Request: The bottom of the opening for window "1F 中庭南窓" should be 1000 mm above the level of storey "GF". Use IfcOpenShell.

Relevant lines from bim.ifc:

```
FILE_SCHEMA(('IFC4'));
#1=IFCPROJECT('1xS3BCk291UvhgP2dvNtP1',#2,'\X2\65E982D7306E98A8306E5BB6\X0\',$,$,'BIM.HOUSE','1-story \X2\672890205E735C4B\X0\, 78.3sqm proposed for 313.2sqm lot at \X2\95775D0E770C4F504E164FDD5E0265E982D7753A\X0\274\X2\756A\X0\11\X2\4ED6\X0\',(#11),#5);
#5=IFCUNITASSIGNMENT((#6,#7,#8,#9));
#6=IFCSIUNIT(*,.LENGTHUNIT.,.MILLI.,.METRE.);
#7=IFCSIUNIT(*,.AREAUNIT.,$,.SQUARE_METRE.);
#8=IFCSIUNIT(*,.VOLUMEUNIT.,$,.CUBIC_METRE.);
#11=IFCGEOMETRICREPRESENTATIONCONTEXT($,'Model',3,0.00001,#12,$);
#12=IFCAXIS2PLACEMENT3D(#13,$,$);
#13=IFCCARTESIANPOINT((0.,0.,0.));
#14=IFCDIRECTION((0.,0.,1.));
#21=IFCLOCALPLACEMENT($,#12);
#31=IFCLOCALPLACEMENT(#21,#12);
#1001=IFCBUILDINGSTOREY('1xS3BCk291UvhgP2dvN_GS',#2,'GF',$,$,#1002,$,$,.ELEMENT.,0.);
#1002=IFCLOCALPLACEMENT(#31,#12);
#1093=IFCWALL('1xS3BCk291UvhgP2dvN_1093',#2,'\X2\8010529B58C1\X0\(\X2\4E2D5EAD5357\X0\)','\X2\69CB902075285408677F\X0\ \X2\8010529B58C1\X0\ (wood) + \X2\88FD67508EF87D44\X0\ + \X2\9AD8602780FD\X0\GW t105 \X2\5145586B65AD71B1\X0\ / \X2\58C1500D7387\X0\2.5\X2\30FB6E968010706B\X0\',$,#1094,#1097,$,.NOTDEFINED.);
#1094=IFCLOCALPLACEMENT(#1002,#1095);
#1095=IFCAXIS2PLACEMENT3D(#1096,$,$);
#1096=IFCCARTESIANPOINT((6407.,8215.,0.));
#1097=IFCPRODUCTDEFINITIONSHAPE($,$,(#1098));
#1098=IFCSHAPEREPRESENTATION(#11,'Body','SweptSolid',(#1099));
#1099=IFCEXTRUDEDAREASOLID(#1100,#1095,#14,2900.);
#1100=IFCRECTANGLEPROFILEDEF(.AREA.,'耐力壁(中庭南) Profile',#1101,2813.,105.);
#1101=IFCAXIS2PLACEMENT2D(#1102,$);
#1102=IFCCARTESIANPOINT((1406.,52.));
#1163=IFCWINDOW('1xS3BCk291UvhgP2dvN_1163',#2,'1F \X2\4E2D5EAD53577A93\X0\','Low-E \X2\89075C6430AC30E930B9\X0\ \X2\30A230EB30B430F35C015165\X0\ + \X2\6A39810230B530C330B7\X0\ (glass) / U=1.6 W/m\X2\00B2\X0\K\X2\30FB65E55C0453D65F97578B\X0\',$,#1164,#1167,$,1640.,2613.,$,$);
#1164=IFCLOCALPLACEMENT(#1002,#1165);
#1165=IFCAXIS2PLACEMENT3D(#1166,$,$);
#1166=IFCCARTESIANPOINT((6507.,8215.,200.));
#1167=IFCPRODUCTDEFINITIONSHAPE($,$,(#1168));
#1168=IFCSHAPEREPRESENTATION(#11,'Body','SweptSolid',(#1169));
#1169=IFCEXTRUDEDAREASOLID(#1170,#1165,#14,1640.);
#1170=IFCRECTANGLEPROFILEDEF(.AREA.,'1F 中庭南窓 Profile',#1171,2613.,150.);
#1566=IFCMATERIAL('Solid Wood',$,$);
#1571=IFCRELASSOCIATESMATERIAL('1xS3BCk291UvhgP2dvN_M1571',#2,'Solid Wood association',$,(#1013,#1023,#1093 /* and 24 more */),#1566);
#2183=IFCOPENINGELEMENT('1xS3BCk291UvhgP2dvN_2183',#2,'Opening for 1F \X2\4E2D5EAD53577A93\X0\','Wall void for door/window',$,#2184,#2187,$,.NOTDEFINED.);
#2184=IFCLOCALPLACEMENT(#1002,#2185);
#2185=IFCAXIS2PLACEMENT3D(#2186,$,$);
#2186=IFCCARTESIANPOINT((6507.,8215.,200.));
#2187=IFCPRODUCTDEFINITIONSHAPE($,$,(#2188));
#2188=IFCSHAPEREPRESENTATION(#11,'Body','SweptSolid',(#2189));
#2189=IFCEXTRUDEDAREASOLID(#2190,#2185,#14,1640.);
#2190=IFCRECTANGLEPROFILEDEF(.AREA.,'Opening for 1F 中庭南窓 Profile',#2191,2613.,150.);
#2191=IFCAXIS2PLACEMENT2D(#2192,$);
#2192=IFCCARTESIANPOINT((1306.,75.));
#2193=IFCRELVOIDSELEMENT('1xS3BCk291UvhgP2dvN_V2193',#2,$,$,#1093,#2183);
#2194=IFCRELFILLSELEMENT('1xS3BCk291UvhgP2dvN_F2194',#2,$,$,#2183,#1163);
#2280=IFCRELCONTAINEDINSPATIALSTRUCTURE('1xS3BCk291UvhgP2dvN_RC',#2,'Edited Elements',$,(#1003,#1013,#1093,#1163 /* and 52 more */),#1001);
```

```python
import numpy as np
import ifcopenshell
import ifcopenshell.api.geometry
import ifcopenshell.geom
import ifcopenshell.util.element
import ifcopenshell.util.placement
import ifcopenshell.util.shape
import ifcopenshell.util.unit

model = ifcopenshell.open("bim.ifc")
unit_scale = ifcopenshell.util.unit.calculate_unit_scale(model)

window = model.by_guid("1xS3BCk291UvhgP2dvN_1163")
opening = window.FillsVoids[0].RelatingOpeningElement
storey = ifcopenshell.util.element.get_container(window, ifc_class="IfcBuildingStorey")
level = ifcopenshell.util.placement.get_local_placement(storey.ObjectPlacement)[2, 3]

# The opening's origin need not be at the sill, so measure its lowest point.
shape = ifcopenshell.geom.create_shape(ifcopenshell.geom.settings(), opening)
bottom = ifcopenshell.util.shape.get_shape_bottom_elevation(shape, shape.geometry) / unit_scale
dz = level + 1 / unit_scale - bottom

shift = np.array([0.0, 0.0, dz])
# The window is not placed relative to its opening, so move both.
for product in (opening, window):
    matrix = ifcopenshell.util.placement.get_local_placement(product.ObjectPlacement)
    matrix[:3, 3] += shift
    ifcopenshell.api.geometry.edit_object_placement(model, product=product, matrix=matrix, is_si=False)

print(f"moved by {dz * unit_scale:+.3f} m")

model.write("bim_v2.ifc")
```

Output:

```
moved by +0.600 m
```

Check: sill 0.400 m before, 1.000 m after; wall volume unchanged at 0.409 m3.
